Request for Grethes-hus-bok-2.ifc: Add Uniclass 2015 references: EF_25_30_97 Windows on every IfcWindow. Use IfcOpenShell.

First a look at what the model holds.

```python
import ifcopenshell

model = ifcopenshell.open("Grethes-hus-bok-2.ifc")
print(model.schema)
print("classifications:", [c.Name for c in model.by_type("IfcClassification")])
for ifc_class in ("IfcDoor", "IfcRoof", "IfcStair", "IfcWall", "IfcWindow"):
    print(ifc_class, len(model.by_type(ifc_class)))
```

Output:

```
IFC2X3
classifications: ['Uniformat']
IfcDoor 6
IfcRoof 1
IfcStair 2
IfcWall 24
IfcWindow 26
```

```python
import ifcopenshell
import ifcopenshell.api.classification

model = ifcopenshell.open("Grethes-hus-bok-2.ifc")

# IFC2X3 requires Source and Edition and has no link from the project to the system.
system = model.create_entity("IfcClassification", Source="NBS", Edition="2015", Name="Uniclass 2015")

codes = {
    "IfcWindow": ("EF_25_30_97", "Windows"),
}
for ifc_class, (code, name) in codes.items():
    products = model.by_type(ifc_class)
    ifcopenshell.api.classification.add_reference(
        model, products=products, classification=system, identification=code, name=name
    )
    print(code, len(products))

model.write("Grethes-hus-bok-2_edited.ifc")
```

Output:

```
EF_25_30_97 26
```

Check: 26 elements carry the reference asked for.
